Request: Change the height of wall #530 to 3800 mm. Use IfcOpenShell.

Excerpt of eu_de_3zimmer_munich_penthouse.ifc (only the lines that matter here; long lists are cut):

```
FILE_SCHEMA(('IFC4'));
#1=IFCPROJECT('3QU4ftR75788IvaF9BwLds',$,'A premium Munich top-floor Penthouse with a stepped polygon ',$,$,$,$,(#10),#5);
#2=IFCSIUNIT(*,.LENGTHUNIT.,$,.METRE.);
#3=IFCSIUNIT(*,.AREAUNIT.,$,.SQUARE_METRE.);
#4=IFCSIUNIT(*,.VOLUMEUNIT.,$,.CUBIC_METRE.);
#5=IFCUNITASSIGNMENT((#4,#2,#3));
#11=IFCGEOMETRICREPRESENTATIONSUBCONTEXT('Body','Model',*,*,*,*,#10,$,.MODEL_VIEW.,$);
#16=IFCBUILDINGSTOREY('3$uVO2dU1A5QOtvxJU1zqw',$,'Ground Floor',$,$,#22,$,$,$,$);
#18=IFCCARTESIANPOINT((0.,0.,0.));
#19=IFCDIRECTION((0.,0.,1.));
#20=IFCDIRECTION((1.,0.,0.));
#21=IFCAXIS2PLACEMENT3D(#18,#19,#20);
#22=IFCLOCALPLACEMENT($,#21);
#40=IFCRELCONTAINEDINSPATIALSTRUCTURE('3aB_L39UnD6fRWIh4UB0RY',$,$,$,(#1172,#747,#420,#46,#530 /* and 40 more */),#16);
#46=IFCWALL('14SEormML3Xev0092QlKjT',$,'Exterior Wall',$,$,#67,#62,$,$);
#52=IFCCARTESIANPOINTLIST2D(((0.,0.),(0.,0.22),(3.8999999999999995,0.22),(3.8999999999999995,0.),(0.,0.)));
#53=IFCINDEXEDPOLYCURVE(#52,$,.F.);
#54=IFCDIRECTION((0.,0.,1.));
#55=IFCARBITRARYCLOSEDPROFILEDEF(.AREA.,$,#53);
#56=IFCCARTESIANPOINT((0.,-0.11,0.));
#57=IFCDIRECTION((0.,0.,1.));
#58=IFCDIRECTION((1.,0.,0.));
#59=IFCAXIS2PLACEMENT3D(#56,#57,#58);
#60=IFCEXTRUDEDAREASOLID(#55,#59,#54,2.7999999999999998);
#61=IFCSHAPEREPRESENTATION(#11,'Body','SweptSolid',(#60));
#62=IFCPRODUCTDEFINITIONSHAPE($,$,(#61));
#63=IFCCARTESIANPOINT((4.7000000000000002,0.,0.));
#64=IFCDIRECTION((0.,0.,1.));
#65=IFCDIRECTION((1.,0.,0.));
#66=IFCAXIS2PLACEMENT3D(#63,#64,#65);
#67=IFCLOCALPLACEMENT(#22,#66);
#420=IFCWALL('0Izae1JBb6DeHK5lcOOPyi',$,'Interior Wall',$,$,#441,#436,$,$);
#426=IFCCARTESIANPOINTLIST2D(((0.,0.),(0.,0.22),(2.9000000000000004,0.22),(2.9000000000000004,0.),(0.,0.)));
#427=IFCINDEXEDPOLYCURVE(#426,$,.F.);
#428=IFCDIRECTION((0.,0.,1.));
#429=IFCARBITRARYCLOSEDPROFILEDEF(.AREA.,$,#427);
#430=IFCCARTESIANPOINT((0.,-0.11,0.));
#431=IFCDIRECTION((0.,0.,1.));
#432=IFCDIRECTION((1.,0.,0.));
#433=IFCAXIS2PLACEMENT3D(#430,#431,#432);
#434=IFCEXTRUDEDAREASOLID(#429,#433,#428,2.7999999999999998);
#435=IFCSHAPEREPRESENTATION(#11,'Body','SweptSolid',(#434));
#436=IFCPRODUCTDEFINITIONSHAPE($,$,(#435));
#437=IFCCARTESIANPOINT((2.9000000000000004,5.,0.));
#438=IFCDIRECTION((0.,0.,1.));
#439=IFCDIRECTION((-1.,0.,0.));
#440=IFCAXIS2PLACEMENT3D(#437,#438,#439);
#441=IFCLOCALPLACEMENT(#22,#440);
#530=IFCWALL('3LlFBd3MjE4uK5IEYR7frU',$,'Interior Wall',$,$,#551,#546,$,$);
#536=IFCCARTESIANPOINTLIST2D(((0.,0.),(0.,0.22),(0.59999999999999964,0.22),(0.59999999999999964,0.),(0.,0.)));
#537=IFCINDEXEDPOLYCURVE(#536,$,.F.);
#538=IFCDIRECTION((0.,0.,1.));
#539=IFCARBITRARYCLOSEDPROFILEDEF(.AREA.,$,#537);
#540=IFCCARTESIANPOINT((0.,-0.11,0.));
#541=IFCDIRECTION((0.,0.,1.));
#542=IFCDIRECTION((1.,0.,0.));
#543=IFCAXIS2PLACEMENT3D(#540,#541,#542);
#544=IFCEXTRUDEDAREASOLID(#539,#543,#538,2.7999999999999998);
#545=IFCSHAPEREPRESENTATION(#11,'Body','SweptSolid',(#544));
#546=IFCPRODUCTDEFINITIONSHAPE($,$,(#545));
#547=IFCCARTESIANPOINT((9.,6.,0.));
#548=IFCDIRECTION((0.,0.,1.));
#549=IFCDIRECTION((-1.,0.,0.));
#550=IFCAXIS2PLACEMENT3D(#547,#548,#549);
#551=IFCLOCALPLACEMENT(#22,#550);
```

```python
import ifcopenshell
import ifcopenshell.geom
import ifcopenshell.util.representation
import ifcopenshell.util.shape
import ifcopenshell.util.unit

model = ifcopenshell.open("eu_de_3zimmer_munich_penthouse.ifc")
unit_scale = ifcopenshell.util.unit.calculate_unit_scale(model)
settings = ifcopenshell.geom.settings()


def volume(element):
    """Net volume in cubic metres, openings subtracted."""
    shape = ifcopenshell.geom.create_shape(settings, element)
    return ifcopenshell.util.shape.get_volume(shape.geometry)


wall = model.by_id(530)
before = volume(wall)

body = ifcopenshell.util.representation.get_representation(wall, "Model", "Body")
solid = body.Items[0]
old_height = solid.Depth
solid.Depth = 3.8 / unit_scale
after = volume(wall)

print(f"height {old_height:g} -> {solid.Depth:g}, volume {before:.3f} -> {after:.3f} m3")

model.write("eu_de_3zimmer_munich_penthouse_v2.ifc")
```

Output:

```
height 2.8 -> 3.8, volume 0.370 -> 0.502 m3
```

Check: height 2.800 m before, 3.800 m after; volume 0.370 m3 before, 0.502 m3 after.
